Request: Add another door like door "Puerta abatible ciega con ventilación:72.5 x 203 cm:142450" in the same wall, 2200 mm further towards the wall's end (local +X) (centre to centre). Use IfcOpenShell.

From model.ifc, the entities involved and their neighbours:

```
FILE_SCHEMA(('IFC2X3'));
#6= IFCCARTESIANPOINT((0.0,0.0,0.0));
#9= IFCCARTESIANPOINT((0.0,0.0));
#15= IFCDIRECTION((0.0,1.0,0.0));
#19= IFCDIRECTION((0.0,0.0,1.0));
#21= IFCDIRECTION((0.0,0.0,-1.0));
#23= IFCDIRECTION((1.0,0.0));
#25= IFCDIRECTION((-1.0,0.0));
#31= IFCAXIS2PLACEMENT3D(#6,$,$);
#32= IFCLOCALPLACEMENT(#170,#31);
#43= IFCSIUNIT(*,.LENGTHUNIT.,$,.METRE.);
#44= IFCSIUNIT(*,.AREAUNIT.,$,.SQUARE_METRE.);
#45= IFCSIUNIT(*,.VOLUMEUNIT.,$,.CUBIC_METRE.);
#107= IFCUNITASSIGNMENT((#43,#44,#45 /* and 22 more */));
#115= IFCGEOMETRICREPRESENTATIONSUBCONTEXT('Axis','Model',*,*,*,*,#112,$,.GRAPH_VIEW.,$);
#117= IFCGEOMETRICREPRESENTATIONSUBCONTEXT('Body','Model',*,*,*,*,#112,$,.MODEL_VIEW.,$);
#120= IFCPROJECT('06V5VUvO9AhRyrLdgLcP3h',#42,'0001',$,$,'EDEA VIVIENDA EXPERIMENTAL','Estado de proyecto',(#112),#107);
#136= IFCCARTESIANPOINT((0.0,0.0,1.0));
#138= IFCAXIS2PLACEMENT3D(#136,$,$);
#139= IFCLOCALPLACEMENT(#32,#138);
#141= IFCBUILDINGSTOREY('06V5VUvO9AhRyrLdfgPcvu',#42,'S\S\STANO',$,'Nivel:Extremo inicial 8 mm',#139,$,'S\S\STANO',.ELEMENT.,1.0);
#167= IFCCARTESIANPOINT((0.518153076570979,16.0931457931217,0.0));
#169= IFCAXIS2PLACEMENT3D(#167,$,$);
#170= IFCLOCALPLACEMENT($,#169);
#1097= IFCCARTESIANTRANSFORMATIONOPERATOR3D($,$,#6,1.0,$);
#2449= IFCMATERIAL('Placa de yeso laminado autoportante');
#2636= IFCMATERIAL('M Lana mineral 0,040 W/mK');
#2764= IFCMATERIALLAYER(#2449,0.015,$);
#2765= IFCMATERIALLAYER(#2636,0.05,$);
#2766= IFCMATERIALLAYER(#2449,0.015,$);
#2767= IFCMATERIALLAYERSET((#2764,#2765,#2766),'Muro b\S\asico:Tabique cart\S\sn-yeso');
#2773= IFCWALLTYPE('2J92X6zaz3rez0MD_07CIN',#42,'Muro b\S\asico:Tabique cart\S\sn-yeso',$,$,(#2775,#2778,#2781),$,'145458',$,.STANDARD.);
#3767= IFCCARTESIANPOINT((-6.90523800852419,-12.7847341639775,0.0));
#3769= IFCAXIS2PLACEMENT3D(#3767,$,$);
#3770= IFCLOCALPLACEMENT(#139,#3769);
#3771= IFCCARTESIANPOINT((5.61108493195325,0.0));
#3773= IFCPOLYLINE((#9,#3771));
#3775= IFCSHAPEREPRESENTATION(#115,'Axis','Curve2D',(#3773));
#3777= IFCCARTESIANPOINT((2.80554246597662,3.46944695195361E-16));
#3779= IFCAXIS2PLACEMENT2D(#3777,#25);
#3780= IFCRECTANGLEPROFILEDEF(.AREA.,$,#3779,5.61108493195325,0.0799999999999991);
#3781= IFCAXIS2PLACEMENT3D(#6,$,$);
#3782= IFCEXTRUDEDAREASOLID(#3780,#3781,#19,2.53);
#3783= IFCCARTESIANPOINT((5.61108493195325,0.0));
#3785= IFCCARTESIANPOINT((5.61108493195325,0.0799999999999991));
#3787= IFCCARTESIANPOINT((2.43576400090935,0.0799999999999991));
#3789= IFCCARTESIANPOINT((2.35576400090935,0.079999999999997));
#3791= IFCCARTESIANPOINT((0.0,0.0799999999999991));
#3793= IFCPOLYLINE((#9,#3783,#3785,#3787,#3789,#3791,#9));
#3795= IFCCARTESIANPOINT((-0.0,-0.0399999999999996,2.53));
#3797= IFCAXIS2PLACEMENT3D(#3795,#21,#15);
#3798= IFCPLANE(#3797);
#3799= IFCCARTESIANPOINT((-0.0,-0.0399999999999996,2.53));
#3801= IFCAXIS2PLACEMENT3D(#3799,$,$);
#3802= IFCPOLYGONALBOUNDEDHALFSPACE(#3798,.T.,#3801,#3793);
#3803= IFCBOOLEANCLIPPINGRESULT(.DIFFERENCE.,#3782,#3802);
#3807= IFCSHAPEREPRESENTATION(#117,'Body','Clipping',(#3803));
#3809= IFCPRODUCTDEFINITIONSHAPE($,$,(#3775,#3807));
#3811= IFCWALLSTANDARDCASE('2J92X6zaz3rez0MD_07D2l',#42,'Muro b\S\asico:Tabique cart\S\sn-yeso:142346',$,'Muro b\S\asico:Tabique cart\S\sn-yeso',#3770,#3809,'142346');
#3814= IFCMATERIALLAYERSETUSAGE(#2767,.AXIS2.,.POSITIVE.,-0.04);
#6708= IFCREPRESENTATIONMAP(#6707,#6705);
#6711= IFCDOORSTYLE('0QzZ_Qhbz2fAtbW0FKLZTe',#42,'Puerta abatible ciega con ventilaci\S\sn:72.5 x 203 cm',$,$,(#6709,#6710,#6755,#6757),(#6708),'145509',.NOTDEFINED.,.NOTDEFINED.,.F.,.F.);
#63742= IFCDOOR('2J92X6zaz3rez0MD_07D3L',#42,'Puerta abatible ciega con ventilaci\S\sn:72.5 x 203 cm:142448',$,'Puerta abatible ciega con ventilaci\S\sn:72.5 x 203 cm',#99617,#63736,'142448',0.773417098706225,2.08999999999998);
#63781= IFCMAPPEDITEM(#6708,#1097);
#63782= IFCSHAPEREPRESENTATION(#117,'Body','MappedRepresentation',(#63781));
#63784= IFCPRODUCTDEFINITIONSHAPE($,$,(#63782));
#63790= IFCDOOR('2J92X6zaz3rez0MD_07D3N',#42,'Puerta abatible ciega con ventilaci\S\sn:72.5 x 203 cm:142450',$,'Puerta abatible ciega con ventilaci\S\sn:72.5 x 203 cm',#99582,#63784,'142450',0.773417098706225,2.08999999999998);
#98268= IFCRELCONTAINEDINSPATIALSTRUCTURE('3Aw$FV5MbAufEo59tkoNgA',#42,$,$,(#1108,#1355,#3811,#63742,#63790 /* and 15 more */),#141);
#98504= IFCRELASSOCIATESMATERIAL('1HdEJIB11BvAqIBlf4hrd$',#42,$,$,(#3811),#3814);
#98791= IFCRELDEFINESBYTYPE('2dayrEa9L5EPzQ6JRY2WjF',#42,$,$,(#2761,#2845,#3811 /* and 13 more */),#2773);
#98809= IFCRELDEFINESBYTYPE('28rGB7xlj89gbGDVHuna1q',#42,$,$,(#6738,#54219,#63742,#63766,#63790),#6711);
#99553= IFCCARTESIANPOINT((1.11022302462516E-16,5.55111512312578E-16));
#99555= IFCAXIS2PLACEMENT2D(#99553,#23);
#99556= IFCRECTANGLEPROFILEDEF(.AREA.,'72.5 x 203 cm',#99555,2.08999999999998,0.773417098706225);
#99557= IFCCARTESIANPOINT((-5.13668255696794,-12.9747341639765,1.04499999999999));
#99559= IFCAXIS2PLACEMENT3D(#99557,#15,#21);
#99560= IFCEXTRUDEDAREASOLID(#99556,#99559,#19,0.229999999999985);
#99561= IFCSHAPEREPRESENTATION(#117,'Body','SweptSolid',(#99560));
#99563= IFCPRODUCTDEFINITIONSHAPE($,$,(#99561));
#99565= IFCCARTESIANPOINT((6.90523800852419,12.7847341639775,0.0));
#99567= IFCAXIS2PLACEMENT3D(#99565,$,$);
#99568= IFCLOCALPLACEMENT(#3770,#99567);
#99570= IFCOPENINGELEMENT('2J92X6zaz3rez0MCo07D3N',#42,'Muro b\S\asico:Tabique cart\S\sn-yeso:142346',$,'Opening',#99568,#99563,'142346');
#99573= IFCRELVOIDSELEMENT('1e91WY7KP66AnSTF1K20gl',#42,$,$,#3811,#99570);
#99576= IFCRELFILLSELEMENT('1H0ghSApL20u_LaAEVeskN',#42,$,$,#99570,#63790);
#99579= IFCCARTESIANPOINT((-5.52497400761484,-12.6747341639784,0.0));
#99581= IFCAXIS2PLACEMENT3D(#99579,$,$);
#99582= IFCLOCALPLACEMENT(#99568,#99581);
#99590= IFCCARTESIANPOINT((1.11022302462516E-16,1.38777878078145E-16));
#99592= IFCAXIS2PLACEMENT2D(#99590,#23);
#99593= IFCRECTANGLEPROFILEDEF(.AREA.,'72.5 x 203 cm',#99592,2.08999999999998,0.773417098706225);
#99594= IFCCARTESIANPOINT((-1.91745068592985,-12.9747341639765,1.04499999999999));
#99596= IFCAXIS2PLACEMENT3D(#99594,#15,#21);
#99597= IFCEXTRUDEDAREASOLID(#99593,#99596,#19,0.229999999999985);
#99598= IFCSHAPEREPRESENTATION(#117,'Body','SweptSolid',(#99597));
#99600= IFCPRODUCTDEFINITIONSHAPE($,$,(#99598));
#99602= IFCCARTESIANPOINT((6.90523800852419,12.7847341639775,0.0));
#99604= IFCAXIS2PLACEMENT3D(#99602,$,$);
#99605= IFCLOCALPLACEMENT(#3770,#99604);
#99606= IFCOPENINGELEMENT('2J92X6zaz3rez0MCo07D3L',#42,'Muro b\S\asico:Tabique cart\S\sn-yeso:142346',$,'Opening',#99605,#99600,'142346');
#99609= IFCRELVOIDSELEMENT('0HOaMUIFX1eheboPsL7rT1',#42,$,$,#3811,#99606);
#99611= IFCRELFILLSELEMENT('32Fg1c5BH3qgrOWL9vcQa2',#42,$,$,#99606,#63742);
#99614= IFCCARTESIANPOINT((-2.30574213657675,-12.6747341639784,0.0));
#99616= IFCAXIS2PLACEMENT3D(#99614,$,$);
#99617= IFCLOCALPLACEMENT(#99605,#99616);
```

```python
import ifcopenshell
import ifcopenshell.api.feature
import ifcopenshell.api.geometry
import ifcopenshell.api.root
import ifcopenshell.geom
import ifcopenshell.util.element
import ifcopenshell.util.placement
import ifcopenshell.util.shape
import ifcopenshell.util.unit

model = ifcopenshell.open("model.ifc")
unit_scale = ifcopenshell.util.unit.calculate_unit_scale(model)
settings = ifcopenshell.geom.settings()


def volume(element):
    """Net volume in cubic metres, openings subtracted."""
    shape = ifcopenshell.geom.create_shape(settings, element)
    return ifcopenshell.util.shape.get_volume(shape.geometry)


def reuse_history(source, copy):
    """copy_class also copies each property set's owner history, people and application; keep the originals."""
    for rel in copy.IsDefinedBy:
        if rel.is_a("IfcRelDefinesByProperties") and (history := rel.RelatingPropertyDefinition.OwnerHistory):
            rel.RelatingPropertyDefinition.OwnerHistory = source.OwnerHistory
            ifcopenshell.util.element.remove_deep2(model, history)


door = model.by_guid("2J92X6zaz3rez0MD_07D3N")
opening = door.FillsVoids[0].RelatingOpeningElement
wall = opening.VoidsElements[0].RelatingBuildingElement
before = volume(wall)
shift = ifcopenshell.util.placement.get_local_placement(wall.ObjectPlacement)[:3, 0] * 2.2 / unit_scale

# copy_class copies the void relationship, type, container and properties, but no geometry.
new_opening = ifcopenshell.api.root.copy_class(model, product=opening)
new_opening.Representation = ifcopenshell.util.element.copy_deep(
    model, opening.Representation, exclude=["IfcGeometricRepresentationContext", "IfcRepresentationMap"]
)
new_opening.Name = "Muro básico:Tabique cartón-yeso"
new_opening.Tag = None
new_door = ifcopenshell.api.root.copy_class(model, product=door)
new_door.Representation = ifcopenshell.util.element.copy_deep(
    model, door.Representation, exclude=["IfcGeometricRepresentationContext", "IfcRepresentationMap"]
)
new_door.Name = "Puerta abatible ciega con ventilación:72.5 x 203 cm"
new_door.Tag = None
reuse_history(door, new_door)
fills = ifcopenshell.api.feature.add_filling(model, opening=new_opening, element=new_door)
fills.OwnerHistory = new_door.OwnerHistory  # required in IFC2X3

for old, new in ((opening, new_opening), (door, new_door)):
    matrix = ifcopenshell.util.placement.get_local_placement(old.ObjectPlacement)
    matrix[:3, 3] += shift
    ifcopenshell.api.geometry.edit_object_placement(model, product=new, matrix=matrix, is_si=False)

after = volume(wall)

print(f"wall volume {before:.3f} -> {after:.3f} m3")

model.write("model-out.ifc")
```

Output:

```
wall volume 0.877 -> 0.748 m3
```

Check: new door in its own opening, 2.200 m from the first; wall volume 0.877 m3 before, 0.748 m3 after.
